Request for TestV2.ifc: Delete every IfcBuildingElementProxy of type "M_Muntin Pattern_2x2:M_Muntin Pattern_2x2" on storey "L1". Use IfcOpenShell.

First a look at what the model holds.

```python
import ifcopenshell
import ifcopenshell.util.element

model = ifcopenshell.open("TestV2.ifc")
print(model.schema)
storey = next(s for s in model.by_type("IfcBuildingStorey") if s.Name == "L1")
proxies = [e for e in ifcopenshell.util.element.get_decomposition(storey) if e.is_a("IfcBuildingElementProxy")]
seen = {}
for e in proxies:
    element_type = ifcopenshell.util.element.get_type(e)
    name = element_type.Name if element_type not in (None, e) else None
    seen[name] = seen.get(name, 0) + 1
for name, count in sorted(seen.items(), key=str):
    print(count, "x", name)
```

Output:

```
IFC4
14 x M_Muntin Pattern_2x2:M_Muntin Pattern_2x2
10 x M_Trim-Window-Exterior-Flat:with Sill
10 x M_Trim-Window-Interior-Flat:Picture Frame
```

```python
import ifcopenshell
import ifcopenshell.api.root
import ifcopenshell.util.element

model = ifcopenshell.open("TestV2.ifc")

storey = next(s for s in model.by_type("IfcBuildingStorey") if s.Name == "L1")
proxies = [e for e in ifcopenshell.util.element.get_decomposition(storey) if e.is_a("IfcBuildingElementProxy")]
targets = [e for e in proxies if (t := ifcopenshell.util.element.get_type(e)) not in (None, e) and t.Name == "M_Muntin Pattern_2x2:M_Muntin Pattern_2x2"]

for e in targets:
    ifcopenshell.api.root.remove_product(model, product=e)
print(len(targets), "removed")

model.write("TestV2_v2.ifc")
```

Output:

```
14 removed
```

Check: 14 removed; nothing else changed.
